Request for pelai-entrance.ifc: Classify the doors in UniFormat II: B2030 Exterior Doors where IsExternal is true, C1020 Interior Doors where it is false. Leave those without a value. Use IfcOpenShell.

First a look at what the model holds.

```python
import ifcopenshell
import ifcopenshell.util.element

model = ifcopenshell.open("pelai-entrance.ifc")
print(model.schema)
print("classifications:", [c.Name for c in model.by_type("IfcClassification")])
values = [ifcopenshell.util.element.get_pset(e, "Pset_DoorCommon", "IsExternal") for e in model.by_type("IfcDoor")]
for value in (True, False, None):
    print("IsExternal", value, values.count(value))
```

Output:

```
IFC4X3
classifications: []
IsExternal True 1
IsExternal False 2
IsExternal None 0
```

```python
import ifcopenshell
import ifcopenshell.api.classification
import ifcopenshell.util.element

model = ifcopenshell.open("pelai-entrance.ifc")

system = ifcopenshell.api.classification.add_classification(model, classification="UniFormat II")

doors = model.by_type("IfcDoor")
external = {e: ifcopenshell.util.element.get_pset(e, "Pset_DoorCommon", "IsExternal") for e in doors}
for flag, code, name in ((True, "B2030", "Exterior Doors"), (False, "C1020", "Interior Doors")):
    products = [e for e in doors if external[e] is flag]
    ifcopenshell.api.classification.add_reference(
        model, products=products, classification=system, identification=code, name=name
    )
    print(code, len(products))

model.write("pelai-entrance_v2.ifc")
```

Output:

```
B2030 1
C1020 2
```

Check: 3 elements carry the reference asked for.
